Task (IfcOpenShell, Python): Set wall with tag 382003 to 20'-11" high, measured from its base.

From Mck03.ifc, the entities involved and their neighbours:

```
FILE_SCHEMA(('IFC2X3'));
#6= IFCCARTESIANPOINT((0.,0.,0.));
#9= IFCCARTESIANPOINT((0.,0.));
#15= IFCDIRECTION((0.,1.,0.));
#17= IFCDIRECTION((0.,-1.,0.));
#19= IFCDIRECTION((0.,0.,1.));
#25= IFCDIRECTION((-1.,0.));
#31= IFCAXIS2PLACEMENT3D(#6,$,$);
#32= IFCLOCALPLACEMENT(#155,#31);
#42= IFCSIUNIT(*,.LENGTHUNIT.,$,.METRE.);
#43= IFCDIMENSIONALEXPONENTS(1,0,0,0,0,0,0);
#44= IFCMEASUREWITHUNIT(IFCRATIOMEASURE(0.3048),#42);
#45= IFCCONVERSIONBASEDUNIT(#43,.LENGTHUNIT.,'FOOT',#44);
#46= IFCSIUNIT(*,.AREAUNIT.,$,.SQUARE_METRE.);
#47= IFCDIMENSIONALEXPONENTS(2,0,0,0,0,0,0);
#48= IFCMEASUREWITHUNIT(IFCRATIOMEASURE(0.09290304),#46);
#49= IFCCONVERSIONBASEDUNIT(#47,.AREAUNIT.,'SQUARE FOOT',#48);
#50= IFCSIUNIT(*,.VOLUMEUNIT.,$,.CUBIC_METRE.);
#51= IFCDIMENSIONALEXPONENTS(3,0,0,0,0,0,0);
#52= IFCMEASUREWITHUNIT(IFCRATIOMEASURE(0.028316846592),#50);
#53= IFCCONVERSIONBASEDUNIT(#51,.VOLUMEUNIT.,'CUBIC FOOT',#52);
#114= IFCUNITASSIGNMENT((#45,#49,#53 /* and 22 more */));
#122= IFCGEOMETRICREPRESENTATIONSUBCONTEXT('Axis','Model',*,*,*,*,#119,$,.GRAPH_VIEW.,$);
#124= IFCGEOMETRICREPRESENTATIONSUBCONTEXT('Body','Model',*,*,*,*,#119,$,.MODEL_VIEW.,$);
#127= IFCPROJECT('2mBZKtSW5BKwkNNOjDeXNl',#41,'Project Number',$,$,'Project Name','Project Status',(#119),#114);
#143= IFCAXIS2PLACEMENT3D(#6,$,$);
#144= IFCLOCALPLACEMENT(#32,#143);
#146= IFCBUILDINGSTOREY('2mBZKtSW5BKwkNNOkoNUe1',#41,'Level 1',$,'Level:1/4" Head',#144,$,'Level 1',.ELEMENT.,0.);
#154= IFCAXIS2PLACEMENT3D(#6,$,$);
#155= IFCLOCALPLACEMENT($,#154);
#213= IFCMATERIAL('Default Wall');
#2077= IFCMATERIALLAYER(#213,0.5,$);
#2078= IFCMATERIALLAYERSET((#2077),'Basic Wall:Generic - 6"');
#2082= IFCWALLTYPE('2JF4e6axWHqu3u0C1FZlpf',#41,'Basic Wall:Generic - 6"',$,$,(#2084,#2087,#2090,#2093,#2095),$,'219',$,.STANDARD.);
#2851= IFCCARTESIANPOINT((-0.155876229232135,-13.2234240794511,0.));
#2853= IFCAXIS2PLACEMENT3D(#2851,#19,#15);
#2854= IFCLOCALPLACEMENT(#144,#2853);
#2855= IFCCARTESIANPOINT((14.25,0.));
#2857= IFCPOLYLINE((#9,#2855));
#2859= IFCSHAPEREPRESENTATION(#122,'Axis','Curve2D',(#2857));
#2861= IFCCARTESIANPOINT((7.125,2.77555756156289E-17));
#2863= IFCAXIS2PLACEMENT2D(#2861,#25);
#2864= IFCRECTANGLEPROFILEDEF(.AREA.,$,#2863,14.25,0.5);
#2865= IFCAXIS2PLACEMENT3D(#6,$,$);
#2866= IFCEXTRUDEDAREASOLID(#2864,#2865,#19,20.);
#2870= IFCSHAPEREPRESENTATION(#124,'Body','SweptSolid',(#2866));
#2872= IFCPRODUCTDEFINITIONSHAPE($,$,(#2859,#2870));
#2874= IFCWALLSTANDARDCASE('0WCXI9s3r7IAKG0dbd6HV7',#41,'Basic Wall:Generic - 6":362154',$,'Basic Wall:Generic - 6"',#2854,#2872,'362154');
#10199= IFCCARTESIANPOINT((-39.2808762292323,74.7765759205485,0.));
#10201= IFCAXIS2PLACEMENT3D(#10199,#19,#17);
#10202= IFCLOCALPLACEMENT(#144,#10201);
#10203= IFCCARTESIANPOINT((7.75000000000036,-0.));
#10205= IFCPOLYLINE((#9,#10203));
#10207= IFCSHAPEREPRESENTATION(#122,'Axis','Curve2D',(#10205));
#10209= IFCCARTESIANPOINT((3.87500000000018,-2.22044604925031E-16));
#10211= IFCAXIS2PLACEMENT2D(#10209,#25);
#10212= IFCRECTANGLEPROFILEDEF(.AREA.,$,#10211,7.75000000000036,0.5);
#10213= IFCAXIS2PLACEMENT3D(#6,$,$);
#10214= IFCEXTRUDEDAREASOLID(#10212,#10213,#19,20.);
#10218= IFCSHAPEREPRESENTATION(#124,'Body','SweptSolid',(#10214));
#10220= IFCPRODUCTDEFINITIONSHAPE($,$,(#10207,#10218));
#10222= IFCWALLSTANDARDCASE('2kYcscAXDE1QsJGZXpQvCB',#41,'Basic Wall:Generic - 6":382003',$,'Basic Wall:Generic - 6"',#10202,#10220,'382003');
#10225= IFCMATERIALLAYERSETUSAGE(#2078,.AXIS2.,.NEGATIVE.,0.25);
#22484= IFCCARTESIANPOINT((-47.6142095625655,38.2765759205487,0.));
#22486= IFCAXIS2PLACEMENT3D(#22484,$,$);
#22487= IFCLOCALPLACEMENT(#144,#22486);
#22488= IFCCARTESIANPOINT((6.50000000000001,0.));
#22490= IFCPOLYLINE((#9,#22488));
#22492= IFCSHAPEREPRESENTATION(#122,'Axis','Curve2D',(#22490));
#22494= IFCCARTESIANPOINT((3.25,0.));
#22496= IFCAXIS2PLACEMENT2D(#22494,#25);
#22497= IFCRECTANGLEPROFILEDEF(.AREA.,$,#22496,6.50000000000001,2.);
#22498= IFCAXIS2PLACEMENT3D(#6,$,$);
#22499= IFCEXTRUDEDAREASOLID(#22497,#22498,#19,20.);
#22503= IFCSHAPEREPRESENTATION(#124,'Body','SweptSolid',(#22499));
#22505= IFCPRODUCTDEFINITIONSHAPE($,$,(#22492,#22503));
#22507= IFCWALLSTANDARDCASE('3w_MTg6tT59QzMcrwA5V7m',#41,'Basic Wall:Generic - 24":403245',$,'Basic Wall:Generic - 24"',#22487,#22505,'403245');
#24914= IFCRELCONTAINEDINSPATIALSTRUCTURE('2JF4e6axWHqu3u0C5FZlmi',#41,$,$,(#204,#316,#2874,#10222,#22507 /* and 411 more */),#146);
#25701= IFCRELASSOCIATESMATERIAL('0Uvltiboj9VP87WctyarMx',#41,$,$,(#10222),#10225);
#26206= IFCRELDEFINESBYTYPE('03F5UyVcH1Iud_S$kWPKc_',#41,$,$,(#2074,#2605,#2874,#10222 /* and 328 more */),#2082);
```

```python
import ifcopenshell
import ifcopenshell.geom
import ifcopenshell.util.representation
import ifcopenshell.util.shape
import ifcopenshell.util.unit

model = ifcopenshell.open("Mck03.ifc")
unit_scale = ifcopenshell.util.unit.calculate_unit_scale(model)
settings = ifcopenshell.geom.settings()


def volume(element):
    """Net volume in cubic metres, openings subtracted."""
    shape = ifcopenshell.geom.create_shape(settings, element)
    return ifcopenshell.util.shape.get_volume(shape.geometry)


wall = model.by_guid("2kYcscAXDE1QsJGZXpQvCB")
before = volume(wall)

body = ifcopenshell.util.representation.get_representation(wall, "Model", "Body")
solid = body.Items[0]
old_height = solid.Depth
solid.Depth = 251 * 0.0254 / unit_scale
after = volume(wall)

print(f"height {old_height:g} -> {solid.Depth:g}, volume {before:.3f} -> {after:.3f} m3")

model.write("Mck03_edited.ifc")
```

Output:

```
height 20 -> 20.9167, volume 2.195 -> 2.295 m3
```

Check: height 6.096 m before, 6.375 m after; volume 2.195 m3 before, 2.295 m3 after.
